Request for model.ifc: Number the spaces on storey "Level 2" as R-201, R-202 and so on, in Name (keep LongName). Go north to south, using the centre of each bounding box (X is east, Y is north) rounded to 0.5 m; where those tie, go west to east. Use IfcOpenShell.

First a look at what the model holds.

```python
import ifcopenshell
import ifcopenshell.util.element
import ifcopenshell.util.placement

model = ifcopenshell.open("model.ifc")
print(model.schema)
storey = next(s for s in model.by_type("IfcBuildingStorey") if s.Name == "Level 2")
spaces = [e for e in ifcopenshell.util.element.get_decomposition(storey) if e.is_a("IfcSpace")]
for e in sorted(spaces, key=lambda e: e.id()):
    origin = ifcopenshell.util.placement.get_local_placement(e.ObjectPlacement)[:3, 3]
    print(e.id(), e.Name, e.LongName, origin.round(2) + 0.0, sep=" | ")
```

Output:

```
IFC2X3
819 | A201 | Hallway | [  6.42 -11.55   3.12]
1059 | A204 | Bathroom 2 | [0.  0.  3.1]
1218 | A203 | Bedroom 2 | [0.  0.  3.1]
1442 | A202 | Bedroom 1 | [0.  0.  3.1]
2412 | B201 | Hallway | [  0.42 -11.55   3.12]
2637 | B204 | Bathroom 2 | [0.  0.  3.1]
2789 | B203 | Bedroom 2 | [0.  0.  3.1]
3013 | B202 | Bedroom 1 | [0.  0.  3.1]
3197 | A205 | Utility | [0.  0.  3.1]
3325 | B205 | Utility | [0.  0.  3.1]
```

```python
import ifcopenshell
import ifcopenshell.geom
import ifcopenshell.util.element
import ifcopenshell.util.shape

model = ifcopenshell.open("model.ifc")
settings = ifcopenshell.geom.settings()
settings.set("use-world-coords", True)


def centre(element):
    shape = ifcopenshell.geom.create_shape(settings, element)
    return ifcopenshell.util.shape.get_bbox_centroid(shape.geometry)


storey = next(s for s in model.by_type("IfcBuildingStorey") if s.Name == "Level 2")
spaces = [e for e in ifcopenshell.util.element.get_decomposition(storey) if e.is_a("IfcSpace")]

# Insertion points can sit at a corner or the storey origin, so sort by the geometry (in metres).
centres = {e: centre(e) for e in spaces}
spaces.sort(key=lambda e: (-round(centres[e][1] / 0.5), centres[e][0]))

for i, e in enumerate(spaces, start=1):
    number = f"R-2{i:02d}"
    e.Name = number
    print(e.id(), number)

model.write("model_v2.ifc")
```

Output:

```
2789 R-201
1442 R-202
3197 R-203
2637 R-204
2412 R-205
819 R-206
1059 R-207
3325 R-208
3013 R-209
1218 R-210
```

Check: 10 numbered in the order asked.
